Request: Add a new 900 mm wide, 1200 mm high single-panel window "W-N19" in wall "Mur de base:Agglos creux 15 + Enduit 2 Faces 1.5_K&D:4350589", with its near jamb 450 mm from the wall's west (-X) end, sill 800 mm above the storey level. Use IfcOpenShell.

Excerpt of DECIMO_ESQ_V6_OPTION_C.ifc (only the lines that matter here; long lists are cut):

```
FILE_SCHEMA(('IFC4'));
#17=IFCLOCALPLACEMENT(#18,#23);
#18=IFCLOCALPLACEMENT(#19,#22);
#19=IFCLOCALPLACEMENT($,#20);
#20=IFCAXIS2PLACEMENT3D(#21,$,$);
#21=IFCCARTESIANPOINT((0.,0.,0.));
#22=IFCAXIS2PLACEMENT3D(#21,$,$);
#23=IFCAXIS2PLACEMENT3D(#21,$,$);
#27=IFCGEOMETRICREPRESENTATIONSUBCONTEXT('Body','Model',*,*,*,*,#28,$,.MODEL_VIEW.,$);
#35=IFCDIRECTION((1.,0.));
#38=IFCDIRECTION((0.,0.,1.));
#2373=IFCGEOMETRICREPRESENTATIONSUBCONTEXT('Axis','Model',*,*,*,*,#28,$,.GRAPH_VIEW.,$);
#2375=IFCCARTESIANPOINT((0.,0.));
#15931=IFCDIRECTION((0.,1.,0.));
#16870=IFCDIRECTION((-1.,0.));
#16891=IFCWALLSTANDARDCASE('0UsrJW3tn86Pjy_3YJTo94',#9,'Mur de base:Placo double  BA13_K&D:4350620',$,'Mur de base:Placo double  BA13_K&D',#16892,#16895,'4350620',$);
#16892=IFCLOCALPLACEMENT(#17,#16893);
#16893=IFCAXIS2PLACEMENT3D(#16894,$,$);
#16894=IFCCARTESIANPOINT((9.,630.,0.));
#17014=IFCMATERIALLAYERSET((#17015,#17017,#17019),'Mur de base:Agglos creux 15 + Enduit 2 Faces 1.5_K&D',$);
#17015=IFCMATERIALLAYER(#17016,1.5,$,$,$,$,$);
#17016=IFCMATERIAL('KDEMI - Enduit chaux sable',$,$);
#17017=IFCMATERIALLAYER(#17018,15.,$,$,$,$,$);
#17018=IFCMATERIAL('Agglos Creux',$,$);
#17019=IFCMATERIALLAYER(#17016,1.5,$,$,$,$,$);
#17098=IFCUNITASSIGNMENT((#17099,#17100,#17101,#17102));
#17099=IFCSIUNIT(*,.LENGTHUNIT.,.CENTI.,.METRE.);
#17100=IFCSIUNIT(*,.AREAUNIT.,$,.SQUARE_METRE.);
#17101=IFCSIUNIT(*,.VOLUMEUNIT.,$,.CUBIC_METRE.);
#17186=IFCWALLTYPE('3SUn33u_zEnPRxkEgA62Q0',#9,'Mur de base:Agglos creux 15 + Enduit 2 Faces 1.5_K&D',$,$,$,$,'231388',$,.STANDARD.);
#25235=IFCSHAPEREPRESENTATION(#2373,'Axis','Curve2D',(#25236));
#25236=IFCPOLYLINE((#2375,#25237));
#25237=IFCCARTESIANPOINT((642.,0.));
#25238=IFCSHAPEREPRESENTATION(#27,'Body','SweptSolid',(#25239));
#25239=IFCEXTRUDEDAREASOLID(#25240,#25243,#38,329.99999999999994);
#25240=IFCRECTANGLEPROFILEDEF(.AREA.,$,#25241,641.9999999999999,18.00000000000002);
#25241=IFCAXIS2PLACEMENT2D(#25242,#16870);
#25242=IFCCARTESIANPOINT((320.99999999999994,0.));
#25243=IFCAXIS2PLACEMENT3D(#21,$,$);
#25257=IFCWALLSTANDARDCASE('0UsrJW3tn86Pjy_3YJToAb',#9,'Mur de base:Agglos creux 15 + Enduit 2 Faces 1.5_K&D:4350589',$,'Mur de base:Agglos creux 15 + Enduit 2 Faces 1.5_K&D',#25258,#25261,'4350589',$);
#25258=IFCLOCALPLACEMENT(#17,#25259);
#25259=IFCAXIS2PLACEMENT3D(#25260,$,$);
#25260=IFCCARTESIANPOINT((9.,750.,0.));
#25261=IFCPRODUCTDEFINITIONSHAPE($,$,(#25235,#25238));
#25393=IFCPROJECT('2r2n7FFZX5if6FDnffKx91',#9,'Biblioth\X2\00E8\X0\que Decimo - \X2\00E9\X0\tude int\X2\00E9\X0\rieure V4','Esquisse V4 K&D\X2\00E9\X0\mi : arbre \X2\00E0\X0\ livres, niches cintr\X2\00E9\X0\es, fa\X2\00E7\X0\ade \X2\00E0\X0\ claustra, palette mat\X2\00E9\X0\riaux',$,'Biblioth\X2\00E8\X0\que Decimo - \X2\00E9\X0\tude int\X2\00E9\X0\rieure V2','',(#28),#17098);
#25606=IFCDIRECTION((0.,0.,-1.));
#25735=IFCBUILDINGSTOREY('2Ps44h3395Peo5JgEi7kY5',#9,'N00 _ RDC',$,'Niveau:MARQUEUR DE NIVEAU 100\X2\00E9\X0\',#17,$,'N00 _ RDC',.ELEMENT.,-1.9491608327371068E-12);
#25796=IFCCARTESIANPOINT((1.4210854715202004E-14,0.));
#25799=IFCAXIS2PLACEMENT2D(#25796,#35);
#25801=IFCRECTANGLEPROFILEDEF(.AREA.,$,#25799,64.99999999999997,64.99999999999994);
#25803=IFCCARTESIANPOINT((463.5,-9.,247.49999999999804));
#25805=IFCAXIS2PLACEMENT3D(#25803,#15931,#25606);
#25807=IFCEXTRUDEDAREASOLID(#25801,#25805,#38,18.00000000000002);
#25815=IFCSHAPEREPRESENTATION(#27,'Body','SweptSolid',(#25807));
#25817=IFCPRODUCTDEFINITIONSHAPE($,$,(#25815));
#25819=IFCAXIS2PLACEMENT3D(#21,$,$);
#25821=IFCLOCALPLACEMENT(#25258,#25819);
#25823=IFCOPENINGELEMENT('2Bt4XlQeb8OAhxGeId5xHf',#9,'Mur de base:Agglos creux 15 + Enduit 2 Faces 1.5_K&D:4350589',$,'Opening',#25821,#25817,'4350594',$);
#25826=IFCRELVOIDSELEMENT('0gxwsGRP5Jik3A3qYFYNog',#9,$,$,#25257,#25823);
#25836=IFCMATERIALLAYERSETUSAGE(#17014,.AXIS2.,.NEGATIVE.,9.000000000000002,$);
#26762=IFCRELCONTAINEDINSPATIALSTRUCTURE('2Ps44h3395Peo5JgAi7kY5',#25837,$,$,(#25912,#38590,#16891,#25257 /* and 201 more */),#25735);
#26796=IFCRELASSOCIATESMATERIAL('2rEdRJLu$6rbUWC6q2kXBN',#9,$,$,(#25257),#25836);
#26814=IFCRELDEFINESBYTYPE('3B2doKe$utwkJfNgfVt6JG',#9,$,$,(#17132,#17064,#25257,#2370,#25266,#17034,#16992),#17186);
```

```python
import numpy as np
import ifcopenshell
import ifcopenshell.api.feature
import ifcopenshell.api.geometry
import ifcopenshell.api.root
import ifcopenshell.api.spatial
import ifcopenshell.geom
import ifcopenshell.util.element
import ifcopenshell.util.placement
import ifcopenshell.util.representation
import ifcopenshell.util.shape
import ifcopenshell.util.unit

model = ifcopenshell.open("DECIMO_ESQ_V6_OPTION_C.ifc")
unit_scale = ifcopenshell.util.unit.calculate_unit_scale(model)
settings = ifcopenshell.geom.settings()


def volume(element):
    """Net volume in cubic metres, openings subtracted."""
    shape = ifcopenshell.geom.create_shape(settings, element)
    return ifcopenshell.util.shape.get_volume(shape.geometry)


wall = model.by_guid("0UsrJW3tn86Pjy_3YJToAb")
storey = ifcopenshell.util.element.get_container(wall, ifc_class="IfcBuildingStorey")
context = ifcopenshell.util.representation.get_context(model, "Model", "Body", "MODEL_VIEW")
before = volume(wall)

width, height, from_end, sill = 0.9, 1.2, 0.45, 0.8  # metres

# The wall runs along its own X axis, and the end named is its -X end.
wall_shape = ifcopenshell.geom.create_shape(settings, wall)
x, y, z = ifcopenshell.util.shape.get_vertices(wall_shape.geometry).T
start = x.min() + from_end
face, thickness = float(y.min()), float(y.max() - y.min())
wall_matrix = ifcopenshell.util.placement.get_local_placement(wall.ObjectPlacement)
level = ifcopenshell.util.placement.get_local_placement(storey.ObjectPlacement)[2, 3]


def in_wall(x, y):
    """Placement at x, y metres in the wall's axes, at sill height."""
    matrix = wall_matrix.copy()
    matrix[:, 3] = wall_matrix @ np.array([x / unit_scale, y / unit_scale, 0.0, 1.0])
    matrix[2, 3] = level + sill / unit_scale
    return matrix


# Opening: a box that overshoots both wall faces by 50 mm.
opening = ifcopenshell.api.root.create_entity(model, ifc_class="IfcOpeningElement", predefined_type="OPENING")
box = ifcopenshell.api.geometry.add_wall_representation(
    model, context=context, length=width, height=height, thickness=thickness + 0.1
)
ifcopenshell.api.geometry.assign_representation(model, product=opening, representation=box)
ifcopenshell.api.geometry.edit_object_placement(model, product=opening, matrix=in_wall(start, face - 0.05), is_si=False)
ifcopenshell.api.feature.add_feature(model, feature=opening, element=wall)

window = ifcopenshell.api.root.create_entity(model, ifc_class="IfcWindow", name="W-N19", predefined_type="WINDOW")
window.OverallWidth, window.OverallHeight = width / unit_scale, height / unit_scale
window.PartitioningType = "SINGLE_PANEL"
body = ifcopenshell.api.geometry.add_window_representation(
    model,
    context=context,
    overall_width=window.OverallWidth,
    overall_height=window.OverallHeight,
    partition_type="SINGLE_PANEL",
)
ifcopenshell.api.geometry.assign_representation(model, product=window, representation=body)
ifcopenshell.api.spatial.assign_container(model, products=[window], relating_structure=storey)
ifcopenshell.api.feature.add_filling(model, opening=opening, element=window)

# Centre the window in the wall's thickness.
ifcopenshell.api.geometry.edit_object_placement(model, product=window, matrix=in_wall(start, face), is_si=False)
window_shape = ifcopenshell.geom.create_shape(settings, window)
depth = ifcopenshell.util.shape.get_vertices(window_shape.geometry)[:, 1]
offset = face + thickness / 2 - (depth.min() + depth.max()) / 2
ifcopenshell.api.geometry.edit_object_placement(model, product=window, matrix=in_wall(start, offset), is_si=False)

after = volume(wall)

print(f"wall volume {before:.3f} -> {after:.3f} m3")

model.write("DECIMO_ESQ_V6_OPTION_C_edited.ifc")
```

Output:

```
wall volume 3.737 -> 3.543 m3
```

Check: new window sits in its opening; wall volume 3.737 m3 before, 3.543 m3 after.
